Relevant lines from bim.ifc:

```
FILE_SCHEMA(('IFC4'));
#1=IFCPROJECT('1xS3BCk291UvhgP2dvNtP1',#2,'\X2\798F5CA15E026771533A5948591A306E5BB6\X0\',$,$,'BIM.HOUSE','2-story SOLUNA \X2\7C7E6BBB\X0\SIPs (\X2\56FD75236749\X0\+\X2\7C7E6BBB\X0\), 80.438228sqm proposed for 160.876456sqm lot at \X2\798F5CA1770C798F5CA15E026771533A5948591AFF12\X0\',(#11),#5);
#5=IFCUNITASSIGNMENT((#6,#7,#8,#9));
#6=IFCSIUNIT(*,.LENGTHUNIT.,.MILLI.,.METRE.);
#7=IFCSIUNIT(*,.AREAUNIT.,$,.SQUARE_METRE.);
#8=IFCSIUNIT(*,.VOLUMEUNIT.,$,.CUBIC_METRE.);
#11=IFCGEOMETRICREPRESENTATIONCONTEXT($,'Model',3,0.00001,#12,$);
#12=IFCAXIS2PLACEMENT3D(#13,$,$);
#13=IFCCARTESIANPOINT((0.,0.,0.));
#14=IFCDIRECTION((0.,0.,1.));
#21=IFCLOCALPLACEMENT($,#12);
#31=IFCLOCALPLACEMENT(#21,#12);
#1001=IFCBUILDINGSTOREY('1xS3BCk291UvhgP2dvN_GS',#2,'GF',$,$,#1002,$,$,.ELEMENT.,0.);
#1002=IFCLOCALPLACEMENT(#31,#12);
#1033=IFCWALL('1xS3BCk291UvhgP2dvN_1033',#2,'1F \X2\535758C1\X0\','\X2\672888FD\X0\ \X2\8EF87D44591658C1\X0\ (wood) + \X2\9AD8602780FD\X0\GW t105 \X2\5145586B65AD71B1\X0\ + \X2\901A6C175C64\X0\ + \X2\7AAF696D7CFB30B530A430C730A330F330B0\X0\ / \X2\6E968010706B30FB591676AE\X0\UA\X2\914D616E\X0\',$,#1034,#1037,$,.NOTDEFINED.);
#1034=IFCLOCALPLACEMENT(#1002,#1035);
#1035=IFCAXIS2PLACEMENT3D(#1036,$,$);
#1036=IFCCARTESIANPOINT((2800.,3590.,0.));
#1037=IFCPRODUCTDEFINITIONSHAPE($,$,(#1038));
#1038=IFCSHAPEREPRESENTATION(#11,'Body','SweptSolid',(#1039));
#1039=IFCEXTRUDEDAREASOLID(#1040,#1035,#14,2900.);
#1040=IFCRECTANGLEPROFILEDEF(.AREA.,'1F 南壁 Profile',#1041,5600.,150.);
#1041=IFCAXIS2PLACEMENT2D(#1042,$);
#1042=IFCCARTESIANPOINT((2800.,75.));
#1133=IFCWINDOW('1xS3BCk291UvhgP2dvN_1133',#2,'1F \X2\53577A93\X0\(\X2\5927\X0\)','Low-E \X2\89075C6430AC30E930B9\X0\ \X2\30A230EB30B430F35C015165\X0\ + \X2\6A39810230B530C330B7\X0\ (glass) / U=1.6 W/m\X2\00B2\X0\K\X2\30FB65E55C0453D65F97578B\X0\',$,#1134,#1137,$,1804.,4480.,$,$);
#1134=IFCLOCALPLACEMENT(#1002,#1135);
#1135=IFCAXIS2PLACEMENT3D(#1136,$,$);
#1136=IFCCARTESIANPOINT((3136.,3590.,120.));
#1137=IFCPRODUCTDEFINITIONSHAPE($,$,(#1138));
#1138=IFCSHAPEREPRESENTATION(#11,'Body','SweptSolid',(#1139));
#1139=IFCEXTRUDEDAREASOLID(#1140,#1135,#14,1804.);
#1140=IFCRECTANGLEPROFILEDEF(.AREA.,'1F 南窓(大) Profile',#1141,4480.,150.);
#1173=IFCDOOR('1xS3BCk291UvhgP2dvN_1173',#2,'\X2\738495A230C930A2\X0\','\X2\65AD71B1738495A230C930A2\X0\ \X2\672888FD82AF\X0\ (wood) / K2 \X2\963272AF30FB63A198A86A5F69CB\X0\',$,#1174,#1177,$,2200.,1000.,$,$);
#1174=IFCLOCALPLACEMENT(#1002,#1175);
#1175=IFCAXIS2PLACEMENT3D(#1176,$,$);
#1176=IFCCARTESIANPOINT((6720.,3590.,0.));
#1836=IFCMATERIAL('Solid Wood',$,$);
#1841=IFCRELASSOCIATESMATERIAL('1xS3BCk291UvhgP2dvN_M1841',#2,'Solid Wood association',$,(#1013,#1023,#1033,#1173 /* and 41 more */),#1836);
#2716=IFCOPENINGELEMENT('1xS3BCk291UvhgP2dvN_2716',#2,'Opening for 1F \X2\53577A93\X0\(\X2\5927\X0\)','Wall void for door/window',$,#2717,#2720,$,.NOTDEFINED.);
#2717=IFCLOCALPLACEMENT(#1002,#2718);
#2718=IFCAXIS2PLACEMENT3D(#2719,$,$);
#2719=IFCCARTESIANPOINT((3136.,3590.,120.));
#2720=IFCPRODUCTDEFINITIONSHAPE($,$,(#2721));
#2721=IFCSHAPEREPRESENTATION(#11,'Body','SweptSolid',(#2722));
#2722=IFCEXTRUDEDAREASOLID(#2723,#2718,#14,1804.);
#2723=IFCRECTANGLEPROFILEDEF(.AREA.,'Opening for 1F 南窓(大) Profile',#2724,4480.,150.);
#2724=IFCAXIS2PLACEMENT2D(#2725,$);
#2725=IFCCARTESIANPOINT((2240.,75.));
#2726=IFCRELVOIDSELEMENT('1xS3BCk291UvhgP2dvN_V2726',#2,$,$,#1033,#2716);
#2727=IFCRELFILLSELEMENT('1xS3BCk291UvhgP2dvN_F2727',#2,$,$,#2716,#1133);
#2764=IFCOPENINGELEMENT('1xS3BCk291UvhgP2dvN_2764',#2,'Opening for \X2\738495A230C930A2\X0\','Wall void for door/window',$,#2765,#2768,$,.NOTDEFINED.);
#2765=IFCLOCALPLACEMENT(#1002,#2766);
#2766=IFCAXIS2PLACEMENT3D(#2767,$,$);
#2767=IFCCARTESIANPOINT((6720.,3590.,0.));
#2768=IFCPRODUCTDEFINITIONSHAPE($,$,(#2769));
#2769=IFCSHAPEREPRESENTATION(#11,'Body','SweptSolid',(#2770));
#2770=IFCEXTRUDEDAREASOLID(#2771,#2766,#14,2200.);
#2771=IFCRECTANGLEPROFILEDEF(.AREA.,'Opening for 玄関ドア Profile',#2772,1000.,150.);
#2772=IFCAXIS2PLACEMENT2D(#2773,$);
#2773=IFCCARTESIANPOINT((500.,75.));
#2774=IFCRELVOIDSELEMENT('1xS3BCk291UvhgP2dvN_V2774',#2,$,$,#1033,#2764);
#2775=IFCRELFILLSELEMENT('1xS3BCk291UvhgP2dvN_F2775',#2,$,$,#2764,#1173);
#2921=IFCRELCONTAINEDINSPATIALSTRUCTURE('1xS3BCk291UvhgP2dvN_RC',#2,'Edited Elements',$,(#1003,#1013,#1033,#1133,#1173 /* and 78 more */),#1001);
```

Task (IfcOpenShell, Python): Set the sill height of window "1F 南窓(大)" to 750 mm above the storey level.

```python
import numpy as np
import ifcopenshell
import ifcopenshell.api.geometry
import ifcopenshell.geom
import ifcopenshell.util.element
import ifcopenshell.util.placement
import ifcopenshell.util.shape
import ifcopenshell.util.unit

model = ifcopenshell.open("bim.ifc")
unit_scale = ifcopenshell.util.unit.calculate_unit_scale(model)

window = model.by_id(1133)
opening = window.FillsVoids[0].RelatingOpeningElement
storey = ifcopenshell.util.element.get_container(window, ifc_class="IfcBuildingStorey")
level = ifcopenshell.util.placement.get_local_placement(storey.ObjectPlacement)[2, 3]

# The opening's origin need not be at the sill, so measure its lowest point.
shape = ifcopenshell.geom.create_shape(ifcopenshell.geom.settings(), opening)
bottom = ifcopenshell.util.shape.get_shape_bottom_elevation(shape, shape.geometry) / unit_scale
dz = level + 0.75 / unit_scale - bottom

shift = np.array([0.0, 0.0, dz])
# The window is not placed relative to its opening, so move both.
for product in (opening, window):
    matrix = ifcopenshell.util.placement.get_local_placement(product.ObjectPlacement)
    matrix[:3, 3] += shift
    ifcopenshell.api.geometry.edit_object_placement(model, product=product, matrix=matrix, is_si=False)

print(f"moved by {dz * unit_scale:+.3f} m")

model.write("bim_edited.ifc")
```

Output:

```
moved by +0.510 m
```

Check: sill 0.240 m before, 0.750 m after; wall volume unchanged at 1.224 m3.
